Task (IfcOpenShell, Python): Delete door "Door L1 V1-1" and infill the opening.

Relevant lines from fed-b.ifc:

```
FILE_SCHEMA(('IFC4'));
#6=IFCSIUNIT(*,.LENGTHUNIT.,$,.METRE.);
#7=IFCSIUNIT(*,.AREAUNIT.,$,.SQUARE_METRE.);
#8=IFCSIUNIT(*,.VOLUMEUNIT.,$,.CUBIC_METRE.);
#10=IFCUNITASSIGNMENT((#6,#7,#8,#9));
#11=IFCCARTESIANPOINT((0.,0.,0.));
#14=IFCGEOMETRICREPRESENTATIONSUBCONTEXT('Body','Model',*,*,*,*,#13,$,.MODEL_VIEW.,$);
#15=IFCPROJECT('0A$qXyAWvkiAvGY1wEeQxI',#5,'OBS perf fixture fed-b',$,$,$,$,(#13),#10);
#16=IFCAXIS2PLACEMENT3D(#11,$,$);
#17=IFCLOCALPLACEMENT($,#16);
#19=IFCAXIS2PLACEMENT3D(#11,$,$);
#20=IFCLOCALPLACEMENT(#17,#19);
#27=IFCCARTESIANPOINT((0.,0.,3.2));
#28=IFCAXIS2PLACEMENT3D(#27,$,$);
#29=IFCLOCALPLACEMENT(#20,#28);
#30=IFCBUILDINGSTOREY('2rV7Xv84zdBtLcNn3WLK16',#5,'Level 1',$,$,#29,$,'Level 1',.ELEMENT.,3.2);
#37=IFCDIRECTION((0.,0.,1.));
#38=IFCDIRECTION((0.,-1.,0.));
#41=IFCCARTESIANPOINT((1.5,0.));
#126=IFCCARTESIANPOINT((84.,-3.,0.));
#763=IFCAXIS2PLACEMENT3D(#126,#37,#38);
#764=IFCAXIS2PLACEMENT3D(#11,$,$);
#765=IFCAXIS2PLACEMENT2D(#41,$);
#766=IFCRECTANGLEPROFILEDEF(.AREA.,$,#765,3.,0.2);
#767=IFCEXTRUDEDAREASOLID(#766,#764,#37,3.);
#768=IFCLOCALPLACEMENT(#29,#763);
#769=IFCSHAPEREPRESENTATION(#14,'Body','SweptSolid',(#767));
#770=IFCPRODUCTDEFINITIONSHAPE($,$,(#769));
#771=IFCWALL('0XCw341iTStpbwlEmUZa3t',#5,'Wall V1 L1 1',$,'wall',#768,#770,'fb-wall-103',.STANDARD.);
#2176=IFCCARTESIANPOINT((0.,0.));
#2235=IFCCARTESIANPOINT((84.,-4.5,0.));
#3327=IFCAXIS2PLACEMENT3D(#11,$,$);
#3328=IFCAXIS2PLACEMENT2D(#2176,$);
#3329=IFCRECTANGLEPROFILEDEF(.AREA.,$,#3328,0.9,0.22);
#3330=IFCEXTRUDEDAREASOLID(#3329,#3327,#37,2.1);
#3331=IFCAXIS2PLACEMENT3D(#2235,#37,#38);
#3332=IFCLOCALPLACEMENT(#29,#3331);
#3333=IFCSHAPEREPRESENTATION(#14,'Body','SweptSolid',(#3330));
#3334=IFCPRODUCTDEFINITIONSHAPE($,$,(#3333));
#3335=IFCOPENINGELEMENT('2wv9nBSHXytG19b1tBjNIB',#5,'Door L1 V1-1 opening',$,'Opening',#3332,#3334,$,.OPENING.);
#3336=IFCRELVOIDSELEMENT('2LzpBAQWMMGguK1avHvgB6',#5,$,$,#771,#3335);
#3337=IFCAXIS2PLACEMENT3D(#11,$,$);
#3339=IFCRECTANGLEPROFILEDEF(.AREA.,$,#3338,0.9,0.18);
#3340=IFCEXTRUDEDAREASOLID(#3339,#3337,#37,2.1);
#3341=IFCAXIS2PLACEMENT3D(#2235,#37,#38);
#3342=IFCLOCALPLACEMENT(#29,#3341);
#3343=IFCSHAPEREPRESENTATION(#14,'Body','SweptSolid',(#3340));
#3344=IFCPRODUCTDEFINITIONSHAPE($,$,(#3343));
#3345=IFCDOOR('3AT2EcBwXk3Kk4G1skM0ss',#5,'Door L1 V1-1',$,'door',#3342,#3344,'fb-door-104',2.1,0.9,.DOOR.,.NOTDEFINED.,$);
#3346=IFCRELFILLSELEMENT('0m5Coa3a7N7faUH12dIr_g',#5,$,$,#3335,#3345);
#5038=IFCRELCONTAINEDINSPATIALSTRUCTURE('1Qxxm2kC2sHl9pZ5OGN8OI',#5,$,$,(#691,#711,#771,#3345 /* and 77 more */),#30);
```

```python
import ifcopenshell
import ifcopenshell.api.feature
import ifcopenshell.api.root
import ifcopenshell.geom
import ifcopenshell.util.shape

model = ifcopenshell.open("fed-b.ifc")
settings = ifcopenshell.geom.settings()


def volume(element):
    """Net volume in cubic metres, openings subtracted."""
    shape = ifcopenshell.geom.create_shape(settings, element)
    return ifcopenshell.util.shape.get_volume(shape.geometry)


door = model.by_guid("3AT2EcBwXk3Kk4G1skM0ss")
opening = door.FillsVoids[0].RelatingOpeningElement
wall = opening.VoidsElements[0].RelatingBuildingElement
before = volume(wall)

ifcopenshell.api.root.remove_product(model, product=door)
ifcopenshell.api.feature.remove_feature(model, feature=opening)

after = volume(wall)

print(f"wall volume {before:.3f} -> {after:.3f} m3")

model.write("fed-b_edited.ifc")
```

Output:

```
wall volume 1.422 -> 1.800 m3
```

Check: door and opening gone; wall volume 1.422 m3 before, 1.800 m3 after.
